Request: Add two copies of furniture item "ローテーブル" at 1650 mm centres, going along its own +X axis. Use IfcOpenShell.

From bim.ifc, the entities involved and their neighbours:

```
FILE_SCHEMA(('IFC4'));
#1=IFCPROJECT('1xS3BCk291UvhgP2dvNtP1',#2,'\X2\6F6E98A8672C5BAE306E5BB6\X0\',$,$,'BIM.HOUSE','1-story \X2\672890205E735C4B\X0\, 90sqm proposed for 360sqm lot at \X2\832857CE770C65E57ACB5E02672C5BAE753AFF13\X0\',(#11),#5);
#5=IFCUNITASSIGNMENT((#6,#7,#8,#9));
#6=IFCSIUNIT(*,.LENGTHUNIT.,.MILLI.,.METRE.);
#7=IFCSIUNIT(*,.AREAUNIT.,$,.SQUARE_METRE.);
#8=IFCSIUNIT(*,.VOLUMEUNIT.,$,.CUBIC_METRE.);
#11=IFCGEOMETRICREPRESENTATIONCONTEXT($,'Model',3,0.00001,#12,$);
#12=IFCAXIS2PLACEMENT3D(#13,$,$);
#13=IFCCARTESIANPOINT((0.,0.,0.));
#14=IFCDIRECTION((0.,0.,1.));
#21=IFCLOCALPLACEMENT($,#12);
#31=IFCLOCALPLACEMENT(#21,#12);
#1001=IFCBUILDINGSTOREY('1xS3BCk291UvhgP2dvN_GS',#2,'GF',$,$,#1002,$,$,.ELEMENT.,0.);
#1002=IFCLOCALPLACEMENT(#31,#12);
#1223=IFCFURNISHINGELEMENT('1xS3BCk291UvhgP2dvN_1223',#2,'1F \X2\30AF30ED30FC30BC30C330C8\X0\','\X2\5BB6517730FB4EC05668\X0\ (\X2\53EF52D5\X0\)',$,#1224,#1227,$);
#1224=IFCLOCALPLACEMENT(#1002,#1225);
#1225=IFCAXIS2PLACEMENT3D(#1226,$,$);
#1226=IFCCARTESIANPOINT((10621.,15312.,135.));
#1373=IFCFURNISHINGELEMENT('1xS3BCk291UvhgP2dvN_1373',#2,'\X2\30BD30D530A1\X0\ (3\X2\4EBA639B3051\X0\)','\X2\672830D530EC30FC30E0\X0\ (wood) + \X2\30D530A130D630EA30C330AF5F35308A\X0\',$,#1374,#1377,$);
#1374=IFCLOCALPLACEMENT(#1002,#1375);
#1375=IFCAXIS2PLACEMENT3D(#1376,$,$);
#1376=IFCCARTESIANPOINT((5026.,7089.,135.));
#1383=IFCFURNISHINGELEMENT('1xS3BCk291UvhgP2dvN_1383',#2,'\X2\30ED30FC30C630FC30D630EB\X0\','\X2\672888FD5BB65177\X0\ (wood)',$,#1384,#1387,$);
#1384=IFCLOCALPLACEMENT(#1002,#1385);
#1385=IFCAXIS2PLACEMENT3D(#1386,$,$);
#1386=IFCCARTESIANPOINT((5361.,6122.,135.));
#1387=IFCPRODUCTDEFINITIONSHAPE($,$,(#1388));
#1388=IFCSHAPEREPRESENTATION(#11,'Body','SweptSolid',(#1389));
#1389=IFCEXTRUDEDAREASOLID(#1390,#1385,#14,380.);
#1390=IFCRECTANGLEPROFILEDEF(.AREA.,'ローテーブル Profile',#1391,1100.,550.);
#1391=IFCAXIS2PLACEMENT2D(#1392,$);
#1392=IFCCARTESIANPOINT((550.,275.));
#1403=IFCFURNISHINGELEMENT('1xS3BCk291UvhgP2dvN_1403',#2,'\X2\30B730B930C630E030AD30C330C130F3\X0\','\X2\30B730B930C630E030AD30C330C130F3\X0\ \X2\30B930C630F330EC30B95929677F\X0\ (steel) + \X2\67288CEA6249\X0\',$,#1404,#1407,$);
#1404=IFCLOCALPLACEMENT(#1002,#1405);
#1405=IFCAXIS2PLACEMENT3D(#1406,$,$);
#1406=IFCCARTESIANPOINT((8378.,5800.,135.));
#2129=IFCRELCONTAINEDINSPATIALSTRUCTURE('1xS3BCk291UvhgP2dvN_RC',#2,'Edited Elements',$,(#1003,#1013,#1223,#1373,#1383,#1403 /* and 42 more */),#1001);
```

```python
import ifcopenshell
import ifcopenshell.api.geometry
import ifcopenshell.api.root
import ifcopenshell.util.element
import ifcopenshell.util.placement

model = ifcopenshell.open("bim.ifc")


def reuse_history(source, copy):
    """copy_class also copies each property set's owner history, people and application; keep the originals."""
    for rel in copy.IsDefinedBy:
        if rel.is_a("IfcRelDefinesByProperties") and (history := rel.RelatingPropertyDefinition.OwnerHistory):
            rel.RelatingPropertyDefinition.OwnerHistory = source.OwnerHistory
            ifcopenshell.util.element.remove_deep2(model, history)


source = model.by_id(1383)
base = ifcopenshell.util.placement.get_local_placement(source.ObjectPlacement)
step = base[:3, 0] * 1650.0

for i in range(1, 3):
    copy = ifcopenshell.api.root.copy_class(model, product=source)
    copy.Representation = ifcopenshell.util.element.copy_deep(
        model, source.Representation, exclude=["IfcGeometricRepresentationContext", "IfcRepresentationMap"]
    )
    reuse_history(source, copy)
    matrix = base.copy()
    matrix[:3, 3] += i * step
    print("added at", matrix[:3, 3].round(3) + 0.0)
    ifcopenshell.api.geometry.edit_object_placement(model, product=copy, matrix=matrix, is_si=False)

model.write("bim_rev.ifc")
```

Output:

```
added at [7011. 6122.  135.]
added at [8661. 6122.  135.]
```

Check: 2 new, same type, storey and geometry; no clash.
